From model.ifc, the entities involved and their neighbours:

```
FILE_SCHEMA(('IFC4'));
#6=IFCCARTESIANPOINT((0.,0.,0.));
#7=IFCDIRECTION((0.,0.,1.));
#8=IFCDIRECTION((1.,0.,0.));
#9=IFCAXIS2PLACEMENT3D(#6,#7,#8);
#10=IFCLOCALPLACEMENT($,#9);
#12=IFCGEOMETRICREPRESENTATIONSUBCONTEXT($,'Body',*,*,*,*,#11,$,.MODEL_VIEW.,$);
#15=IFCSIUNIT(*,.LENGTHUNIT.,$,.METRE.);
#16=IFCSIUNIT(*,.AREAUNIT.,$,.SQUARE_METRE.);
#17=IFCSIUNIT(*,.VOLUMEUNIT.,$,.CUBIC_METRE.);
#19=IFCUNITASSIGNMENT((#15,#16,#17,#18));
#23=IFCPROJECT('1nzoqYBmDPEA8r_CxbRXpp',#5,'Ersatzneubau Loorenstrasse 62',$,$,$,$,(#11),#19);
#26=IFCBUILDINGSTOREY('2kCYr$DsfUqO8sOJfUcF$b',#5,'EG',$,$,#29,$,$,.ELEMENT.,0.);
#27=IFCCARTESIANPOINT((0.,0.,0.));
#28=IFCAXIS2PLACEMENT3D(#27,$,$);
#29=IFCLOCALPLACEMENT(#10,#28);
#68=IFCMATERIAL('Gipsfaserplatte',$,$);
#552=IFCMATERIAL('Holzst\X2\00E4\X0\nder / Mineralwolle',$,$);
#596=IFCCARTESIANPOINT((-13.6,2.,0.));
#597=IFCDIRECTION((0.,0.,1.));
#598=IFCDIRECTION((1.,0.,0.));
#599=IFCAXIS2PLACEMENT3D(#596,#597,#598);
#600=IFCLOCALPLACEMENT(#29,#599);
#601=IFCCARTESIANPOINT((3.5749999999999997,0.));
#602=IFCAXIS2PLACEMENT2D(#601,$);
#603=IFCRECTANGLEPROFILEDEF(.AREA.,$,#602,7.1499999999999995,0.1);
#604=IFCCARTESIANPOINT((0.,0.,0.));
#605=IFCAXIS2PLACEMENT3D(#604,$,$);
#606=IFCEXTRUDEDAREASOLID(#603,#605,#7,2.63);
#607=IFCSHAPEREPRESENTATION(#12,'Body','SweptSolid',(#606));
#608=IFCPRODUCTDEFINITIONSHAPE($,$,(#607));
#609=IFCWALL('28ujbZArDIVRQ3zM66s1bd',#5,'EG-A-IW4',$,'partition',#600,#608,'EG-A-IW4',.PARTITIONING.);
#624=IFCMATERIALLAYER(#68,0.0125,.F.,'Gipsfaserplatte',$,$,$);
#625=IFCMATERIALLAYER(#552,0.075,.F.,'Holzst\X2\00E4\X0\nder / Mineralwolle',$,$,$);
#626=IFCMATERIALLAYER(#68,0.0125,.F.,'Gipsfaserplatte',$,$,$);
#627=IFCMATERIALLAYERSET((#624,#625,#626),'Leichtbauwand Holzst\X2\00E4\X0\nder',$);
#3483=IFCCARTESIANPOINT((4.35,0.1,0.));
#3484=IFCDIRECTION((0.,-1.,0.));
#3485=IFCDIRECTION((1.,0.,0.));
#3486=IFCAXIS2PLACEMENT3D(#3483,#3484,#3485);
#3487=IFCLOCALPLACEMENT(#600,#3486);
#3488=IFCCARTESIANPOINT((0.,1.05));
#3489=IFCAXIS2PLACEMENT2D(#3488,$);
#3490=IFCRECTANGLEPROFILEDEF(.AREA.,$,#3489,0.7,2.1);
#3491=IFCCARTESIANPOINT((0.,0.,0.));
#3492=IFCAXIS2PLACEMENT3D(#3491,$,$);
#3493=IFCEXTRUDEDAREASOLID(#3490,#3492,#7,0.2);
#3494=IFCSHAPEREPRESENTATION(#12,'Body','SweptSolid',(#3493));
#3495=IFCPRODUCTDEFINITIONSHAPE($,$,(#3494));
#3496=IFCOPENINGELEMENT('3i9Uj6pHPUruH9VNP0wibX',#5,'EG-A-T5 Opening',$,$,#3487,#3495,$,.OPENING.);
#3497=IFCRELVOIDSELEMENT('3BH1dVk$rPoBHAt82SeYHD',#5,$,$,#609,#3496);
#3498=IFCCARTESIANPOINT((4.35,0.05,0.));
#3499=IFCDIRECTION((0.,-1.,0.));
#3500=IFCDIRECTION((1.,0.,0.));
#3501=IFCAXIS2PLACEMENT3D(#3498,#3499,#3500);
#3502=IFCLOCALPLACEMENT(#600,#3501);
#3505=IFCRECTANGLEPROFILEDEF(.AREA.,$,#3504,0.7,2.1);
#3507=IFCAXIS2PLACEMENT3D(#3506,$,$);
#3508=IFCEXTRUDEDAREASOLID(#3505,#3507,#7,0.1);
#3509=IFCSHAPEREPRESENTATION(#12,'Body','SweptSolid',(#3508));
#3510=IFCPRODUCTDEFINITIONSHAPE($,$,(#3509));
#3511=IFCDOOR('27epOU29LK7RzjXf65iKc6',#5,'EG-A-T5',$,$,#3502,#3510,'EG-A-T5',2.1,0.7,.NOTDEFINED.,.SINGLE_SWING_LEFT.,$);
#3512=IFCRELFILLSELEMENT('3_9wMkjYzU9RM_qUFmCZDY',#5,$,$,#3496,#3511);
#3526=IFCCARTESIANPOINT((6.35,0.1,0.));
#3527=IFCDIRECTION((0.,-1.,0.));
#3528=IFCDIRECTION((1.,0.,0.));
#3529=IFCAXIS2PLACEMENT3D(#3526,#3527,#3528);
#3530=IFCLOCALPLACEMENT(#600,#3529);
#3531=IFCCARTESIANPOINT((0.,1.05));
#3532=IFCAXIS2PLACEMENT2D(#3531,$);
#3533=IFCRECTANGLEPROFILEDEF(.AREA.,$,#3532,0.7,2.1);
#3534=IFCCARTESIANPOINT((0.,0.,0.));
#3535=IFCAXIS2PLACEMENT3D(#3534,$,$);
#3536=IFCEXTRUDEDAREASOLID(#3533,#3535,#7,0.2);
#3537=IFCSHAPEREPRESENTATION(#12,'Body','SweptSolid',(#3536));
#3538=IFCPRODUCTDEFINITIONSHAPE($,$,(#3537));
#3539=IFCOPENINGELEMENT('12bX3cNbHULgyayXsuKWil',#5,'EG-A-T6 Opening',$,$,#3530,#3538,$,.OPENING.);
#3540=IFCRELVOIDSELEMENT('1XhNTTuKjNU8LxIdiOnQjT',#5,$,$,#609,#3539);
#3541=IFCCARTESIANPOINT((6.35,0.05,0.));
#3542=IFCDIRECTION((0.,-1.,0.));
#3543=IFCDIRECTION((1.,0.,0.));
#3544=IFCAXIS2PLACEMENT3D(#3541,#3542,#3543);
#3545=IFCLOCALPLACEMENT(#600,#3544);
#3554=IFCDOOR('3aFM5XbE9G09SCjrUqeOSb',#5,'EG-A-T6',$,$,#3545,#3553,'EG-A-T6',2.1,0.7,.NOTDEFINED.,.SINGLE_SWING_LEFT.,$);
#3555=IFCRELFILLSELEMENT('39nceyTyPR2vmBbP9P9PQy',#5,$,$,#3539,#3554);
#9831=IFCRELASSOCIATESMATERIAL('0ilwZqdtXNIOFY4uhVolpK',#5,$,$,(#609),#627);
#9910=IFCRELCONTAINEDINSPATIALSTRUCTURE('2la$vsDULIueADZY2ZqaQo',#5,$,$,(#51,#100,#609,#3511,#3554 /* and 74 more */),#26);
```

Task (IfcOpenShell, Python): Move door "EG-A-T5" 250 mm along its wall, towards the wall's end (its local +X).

```python
import ifcopenshell
import ifcopenshell.api.geometry
import ifcopenshell.util.placement

model = ifcopenshell.open("model.ifc")

door = model.by_id(3511)
opening = door.FillsVoids[0].RelatingOpeningElement
wall = opening.VoidsElements[0].RelatingBuildingElement

wall_matrix = ifcopenshell.util.placement.get_local_placement(wall.ObjectPlacement)
shift = wall_matrix[:3, 0] * 0.25
before = ifcopenshell.util.placement.get_local_placement(door.ObjectPlacement)[:3, 3].copy()

# The door is not placed relative to its opening, so move both.
for product in (opening, door):
    matrix = ifcopenshell.util.placement.get_local_placement(product.ObjectPlacement)
    matrix[:3, 3] += shift
    ifcopenshell.api.geometry.edit_object_placement(model, product=product, matrix=matrix, is_si=False)

after = ifcopenshell.util.placement.get_local_placement(door.ObjectPlacement)[:3, 3]
print("door moved by", (after - before).round(3) + 0.0)

model.write("model_edited.ifc")
```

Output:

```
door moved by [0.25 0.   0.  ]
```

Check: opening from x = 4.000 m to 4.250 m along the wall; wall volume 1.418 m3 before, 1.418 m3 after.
